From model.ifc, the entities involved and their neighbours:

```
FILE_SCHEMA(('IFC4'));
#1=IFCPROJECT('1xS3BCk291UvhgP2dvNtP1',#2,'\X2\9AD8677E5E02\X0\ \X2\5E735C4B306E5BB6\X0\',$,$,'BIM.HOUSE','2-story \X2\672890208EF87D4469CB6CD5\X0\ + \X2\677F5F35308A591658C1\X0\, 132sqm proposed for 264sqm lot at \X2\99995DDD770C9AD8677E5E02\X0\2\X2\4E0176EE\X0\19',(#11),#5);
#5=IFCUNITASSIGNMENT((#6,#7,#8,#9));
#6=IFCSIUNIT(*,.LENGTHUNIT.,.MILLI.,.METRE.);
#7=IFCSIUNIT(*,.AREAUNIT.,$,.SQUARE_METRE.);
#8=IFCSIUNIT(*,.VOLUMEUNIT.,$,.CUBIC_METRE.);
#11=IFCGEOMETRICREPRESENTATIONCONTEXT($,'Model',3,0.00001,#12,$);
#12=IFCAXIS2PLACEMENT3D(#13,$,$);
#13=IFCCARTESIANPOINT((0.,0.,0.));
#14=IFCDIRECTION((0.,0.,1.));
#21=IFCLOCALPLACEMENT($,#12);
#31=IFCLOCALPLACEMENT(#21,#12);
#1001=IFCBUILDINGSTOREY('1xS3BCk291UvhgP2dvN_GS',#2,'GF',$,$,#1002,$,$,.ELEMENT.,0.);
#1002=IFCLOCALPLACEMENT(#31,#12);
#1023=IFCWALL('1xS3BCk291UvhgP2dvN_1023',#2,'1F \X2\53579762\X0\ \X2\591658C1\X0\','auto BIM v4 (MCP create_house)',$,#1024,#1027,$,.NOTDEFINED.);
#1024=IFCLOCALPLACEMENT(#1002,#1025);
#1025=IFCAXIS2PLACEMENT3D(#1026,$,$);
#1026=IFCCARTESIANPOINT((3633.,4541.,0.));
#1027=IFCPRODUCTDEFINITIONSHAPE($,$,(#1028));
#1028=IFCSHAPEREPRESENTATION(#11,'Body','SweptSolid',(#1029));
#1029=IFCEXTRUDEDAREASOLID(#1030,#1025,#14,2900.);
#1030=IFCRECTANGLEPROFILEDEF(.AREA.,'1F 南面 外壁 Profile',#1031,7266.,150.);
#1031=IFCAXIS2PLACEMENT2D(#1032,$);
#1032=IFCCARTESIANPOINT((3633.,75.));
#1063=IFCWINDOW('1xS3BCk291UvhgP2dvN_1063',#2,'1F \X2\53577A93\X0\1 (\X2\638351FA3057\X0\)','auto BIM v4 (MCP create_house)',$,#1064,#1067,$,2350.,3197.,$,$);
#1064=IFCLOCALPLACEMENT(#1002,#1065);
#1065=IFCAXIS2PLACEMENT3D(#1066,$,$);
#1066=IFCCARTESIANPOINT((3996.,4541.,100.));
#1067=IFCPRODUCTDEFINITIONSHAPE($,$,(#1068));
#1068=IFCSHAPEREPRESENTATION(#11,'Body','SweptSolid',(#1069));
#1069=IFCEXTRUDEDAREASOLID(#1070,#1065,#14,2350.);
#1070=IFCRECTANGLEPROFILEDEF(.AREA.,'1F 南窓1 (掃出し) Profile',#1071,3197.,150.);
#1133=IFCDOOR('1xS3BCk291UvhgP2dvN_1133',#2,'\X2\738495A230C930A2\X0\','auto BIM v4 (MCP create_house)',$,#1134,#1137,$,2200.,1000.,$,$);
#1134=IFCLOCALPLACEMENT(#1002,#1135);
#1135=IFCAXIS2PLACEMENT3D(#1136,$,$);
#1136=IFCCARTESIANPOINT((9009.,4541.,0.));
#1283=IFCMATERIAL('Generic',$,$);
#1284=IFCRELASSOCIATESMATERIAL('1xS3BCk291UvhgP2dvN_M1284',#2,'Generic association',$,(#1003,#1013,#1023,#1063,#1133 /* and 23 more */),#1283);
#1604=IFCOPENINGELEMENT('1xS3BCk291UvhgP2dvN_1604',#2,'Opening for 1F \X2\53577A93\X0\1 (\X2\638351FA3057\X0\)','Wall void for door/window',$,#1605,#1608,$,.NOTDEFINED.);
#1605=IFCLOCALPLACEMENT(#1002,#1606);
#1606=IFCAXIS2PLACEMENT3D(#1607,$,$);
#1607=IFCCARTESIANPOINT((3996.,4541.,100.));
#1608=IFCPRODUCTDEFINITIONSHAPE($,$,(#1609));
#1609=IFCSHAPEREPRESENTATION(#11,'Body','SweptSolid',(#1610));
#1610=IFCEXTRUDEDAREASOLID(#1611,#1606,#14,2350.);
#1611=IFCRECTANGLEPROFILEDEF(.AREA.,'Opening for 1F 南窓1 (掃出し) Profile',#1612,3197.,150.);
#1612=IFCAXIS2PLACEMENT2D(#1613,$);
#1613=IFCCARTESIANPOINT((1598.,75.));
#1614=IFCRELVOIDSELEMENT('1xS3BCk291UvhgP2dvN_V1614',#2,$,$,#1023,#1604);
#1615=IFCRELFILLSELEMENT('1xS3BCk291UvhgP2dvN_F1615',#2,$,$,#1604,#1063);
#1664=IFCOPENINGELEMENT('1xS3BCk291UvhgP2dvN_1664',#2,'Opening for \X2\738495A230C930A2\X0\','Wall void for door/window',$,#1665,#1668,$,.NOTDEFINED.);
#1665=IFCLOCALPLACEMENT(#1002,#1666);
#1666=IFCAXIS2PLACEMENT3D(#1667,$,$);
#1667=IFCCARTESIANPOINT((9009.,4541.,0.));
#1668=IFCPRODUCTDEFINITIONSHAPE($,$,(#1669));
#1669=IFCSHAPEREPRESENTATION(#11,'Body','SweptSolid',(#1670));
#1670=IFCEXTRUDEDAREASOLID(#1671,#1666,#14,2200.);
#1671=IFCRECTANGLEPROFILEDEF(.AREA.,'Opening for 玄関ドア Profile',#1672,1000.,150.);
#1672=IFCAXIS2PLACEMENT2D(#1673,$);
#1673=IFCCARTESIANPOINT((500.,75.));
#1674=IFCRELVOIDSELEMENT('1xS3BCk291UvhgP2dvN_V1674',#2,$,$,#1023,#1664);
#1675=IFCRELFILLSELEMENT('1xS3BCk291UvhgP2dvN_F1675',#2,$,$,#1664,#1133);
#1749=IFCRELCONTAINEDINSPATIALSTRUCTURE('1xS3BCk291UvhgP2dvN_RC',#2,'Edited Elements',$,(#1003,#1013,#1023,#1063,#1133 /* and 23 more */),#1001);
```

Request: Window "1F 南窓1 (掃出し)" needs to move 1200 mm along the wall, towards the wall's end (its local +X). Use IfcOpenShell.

```python
import ifcopenshell
import ifcopenshell.api.geometry
import ifcopenshell.util.placement

model = ifcopenshell.open("model.ifc")

window = model.by_id(1063)
opening = window.FillsVoids[0].RelatingOpeningElement
wall = opening.VoidsElements[0].RelatingBuildingElement

wall_matrix = ifcopenshell.util.placement.get_local_placement(wall.ObjectPlacement)
shift = wall_matrix[:3, 0] * 1200.0
before = ifcopenshell.util.placement.get_local_placement(window.ObjectPlacement)[:3, 3].copy()

# The window is not placed relative to its opening, so move both.
for product in (opening, window):
    matrix = ifcopenshell.util.placement.get_local_placement(product.ObjectPlacement)
    matrix[:3, 3] += shift
    ifcopenshell.api.geometry.edit_object_placement(model, product=product, matrix=matrix, is_si=False)

after = ifcopenshell.util.placement.get_local_placement(window.ObjectPlacement)[:3, 3]
print("window moved by", (after - before).round(3) + 0.0)

model.write("model_rev.ifc")
```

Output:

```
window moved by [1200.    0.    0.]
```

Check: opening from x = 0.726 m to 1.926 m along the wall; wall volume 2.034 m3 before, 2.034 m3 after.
